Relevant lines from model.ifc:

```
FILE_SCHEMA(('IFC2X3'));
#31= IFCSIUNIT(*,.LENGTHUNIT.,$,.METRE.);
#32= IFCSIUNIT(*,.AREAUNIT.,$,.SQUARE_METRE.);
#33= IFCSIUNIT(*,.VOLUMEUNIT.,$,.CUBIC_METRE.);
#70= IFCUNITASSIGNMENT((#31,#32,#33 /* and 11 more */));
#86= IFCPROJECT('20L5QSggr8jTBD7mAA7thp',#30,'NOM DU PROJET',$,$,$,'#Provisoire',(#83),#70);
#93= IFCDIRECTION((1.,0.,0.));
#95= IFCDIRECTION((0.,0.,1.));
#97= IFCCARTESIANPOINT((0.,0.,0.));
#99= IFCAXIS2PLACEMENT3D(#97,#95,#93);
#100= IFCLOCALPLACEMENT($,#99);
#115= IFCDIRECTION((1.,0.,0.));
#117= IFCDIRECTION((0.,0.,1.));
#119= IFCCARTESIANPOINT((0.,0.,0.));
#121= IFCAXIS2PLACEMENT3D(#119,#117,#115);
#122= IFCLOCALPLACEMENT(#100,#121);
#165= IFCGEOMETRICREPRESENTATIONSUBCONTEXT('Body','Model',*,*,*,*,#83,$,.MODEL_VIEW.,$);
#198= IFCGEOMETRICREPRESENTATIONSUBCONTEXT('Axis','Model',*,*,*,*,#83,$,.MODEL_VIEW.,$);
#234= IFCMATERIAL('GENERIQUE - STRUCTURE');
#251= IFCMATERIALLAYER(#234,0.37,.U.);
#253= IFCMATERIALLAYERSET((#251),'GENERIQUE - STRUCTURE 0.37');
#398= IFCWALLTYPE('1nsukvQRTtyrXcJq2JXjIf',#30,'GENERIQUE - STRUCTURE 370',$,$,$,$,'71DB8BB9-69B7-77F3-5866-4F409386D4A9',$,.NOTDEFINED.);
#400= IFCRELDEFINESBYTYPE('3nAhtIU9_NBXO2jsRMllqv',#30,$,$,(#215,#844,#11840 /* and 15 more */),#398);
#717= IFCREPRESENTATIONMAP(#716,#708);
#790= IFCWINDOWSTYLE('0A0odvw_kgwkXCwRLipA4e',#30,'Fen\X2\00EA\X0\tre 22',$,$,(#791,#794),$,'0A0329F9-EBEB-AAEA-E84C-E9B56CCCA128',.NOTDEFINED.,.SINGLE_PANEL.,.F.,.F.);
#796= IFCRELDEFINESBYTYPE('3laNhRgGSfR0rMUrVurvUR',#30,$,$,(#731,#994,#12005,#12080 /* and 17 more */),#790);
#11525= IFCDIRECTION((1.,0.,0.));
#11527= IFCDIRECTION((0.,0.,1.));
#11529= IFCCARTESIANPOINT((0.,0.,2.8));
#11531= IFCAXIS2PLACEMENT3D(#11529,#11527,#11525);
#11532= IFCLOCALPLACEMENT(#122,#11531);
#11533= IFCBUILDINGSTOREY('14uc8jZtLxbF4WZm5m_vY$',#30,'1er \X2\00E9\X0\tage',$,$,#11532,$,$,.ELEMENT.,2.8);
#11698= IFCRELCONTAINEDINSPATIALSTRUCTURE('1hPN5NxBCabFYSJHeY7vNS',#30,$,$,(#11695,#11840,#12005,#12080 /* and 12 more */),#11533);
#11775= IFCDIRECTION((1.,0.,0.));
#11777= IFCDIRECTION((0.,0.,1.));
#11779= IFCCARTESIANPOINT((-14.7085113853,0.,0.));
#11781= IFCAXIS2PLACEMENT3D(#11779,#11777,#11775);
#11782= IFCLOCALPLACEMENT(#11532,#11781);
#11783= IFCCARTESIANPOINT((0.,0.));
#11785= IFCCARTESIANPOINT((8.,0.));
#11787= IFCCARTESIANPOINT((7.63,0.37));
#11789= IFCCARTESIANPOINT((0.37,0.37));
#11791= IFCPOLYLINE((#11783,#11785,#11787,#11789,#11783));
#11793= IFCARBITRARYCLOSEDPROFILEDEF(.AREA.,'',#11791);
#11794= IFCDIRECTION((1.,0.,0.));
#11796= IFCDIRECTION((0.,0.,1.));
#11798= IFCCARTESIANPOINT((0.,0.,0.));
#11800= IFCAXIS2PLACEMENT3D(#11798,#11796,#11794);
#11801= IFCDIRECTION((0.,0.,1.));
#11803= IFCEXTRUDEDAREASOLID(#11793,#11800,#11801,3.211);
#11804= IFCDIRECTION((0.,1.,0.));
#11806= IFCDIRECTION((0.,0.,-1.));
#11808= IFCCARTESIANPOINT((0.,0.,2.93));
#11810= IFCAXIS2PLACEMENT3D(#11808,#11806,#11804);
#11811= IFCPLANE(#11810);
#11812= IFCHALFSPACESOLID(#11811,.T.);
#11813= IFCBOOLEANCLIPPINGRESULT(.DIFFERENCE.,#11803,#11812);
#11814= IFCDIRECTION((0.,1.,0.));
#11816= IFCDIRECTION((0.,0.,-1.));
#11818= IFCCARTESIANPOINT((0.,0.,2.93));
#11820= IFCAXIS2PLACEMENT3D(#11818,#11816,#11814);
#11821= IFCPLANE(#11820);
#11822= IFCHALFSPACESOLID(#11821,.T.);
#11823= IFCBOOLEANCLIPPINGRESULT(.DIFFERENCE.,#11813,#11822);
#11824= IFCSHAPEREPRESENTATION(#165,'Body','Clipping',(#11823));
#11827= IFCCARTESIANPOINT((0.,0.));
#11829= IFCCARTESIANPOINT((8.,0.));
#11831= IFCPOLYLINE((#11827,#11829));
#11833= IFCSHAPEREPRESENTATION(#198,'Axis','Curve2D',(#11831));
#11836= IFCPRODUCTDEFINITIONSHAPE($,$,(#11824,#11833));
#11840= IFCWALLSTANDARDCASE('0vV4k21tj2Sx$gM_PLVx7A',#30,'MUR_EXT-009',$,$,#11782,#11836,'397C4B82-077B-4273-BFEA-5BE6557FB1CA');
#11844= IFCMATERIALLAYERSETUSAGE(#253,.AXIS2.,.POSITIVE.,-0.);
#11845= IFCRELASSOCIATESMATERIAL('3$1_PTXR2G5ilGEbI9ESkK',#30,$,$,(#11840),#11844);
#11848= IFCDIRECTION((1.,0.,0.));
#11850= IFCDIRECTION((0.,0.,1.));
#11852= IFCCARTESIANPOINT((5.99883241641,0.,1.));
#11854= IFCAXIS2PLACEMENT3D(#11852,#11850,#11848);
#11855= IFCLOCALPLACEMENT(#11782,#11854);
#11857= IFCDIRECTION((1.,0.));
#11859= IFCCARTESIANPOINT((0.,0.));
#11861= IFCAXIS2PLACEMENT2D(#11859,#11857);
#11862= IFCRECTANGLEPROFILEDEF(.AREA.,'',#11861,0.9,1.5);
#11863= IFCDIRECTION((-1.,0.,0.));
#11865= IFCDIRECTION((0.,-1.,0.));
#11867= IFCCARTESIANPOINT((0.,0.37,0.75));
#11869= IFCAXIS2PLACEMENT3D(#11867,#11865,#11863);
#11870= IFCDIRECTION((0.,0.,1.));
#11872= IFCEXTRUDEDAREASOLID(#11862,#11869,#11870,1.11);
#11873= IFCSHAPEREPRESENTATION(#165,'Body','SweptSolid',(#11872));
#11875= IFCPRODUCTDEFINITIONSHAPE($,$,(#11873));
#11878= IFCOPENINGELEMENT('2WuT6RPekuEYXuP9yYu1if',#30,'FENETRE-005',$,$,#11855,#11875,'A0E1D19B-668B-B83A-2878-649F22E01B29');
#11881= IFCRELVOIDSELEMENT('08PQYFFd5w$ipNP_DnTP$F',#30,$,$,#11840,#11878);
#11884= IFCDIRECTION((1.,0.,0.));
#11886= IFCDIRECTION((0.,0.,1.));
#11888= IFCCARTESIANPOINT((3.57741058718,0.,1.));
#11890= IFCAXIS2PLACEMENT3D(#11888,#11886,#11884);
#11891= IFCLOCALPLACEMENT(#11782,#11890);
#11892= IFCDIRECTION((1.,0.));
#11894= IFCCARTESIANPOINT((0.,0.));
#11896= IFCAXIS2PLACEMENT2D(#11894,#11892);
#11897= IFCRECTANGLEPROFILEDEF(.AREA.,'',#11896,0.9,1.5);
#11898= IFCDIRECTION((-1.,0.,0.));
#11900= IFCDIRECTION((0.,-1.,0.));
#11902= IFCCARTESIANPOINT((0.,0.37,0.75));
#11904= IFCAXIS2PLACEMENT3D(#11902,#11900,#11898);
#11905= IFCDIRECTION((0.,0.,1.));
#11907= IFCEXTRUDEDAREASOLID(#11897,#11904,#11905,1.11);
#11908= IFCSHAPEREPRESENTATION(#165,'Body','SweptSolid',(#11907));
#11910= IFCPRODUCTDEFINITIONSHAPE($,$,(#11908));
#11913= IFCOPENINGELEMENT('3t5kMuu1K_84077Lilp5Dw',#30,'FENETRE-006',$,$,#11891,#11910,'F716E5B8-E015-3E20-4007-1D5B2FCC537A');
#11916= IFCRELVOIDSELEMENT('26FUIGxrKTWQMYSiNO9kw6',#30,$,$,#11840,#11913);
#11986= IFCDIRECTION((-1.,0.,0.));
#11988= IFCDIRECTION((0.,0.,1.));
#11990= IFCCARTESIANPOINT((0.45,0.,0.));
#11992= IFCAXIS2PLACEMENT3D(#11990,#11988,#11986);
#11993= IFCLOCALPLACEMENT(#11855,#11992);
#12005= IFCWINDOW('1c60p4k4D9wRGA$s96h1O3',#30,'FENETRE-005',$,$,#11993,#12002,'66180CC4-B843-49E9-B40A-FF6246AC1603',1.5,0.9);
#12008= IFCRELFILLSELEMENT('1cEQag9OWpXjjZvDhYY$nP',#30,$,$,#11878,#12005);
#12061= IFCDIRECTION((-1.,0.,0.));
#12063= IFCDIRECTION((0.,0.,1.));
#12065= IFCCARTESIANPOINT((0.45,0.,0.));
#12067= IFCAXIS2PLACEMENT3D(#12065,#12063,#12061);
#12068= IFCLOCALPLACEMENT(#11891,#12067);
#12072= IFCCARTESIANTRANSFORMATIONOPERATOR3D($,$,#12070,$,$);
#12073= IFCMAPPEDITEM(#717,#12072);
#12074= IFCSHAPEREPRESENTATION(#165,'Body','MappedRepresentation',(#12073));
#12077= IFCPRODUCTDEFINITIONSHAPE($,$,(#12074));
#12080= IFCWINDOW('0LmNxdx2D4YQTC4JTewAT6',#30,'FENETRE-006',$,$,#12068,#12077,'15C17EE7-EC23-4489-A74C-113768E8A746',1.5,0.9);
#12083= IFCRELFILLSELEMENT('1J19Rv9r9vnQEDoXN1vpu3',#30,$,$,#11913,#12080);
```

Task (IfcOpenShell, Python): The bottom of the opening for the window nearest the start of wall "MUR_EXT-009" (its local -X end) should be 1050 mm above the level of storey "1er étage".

```python
import numpy as np
import ifcopenshell
import ifcopenshell.api.geometry
import ifcopenshell.geom
import ifcopenshell.util.element
import ifcopenshell.util.placement
import ifcopenshell.util.shape
import ifcopenshell.util.unit

model = ifcopenshell.open("model.ifc")
unit_scale = ifcopenshell.util.unit.calculate_unit_scale(model)

window = model.by_id(12080)
opening = window.FillsVoids[0].RelatingOpeningElement
storey = ifcopenshell.util.element.get_container(window, ifc_class="IfcBuildingStorey")
level = ifcopenshell.util.placement.get_local_placement(storey.ObjectPlacement)[2, 3]

# The opening's origin need not be at the sill, so measure its lowest point.
shape = ifcopenshell.geom.create_shape(ifcopenshell.geom.settings(), opening)
bottom = ifcopenshell.util.shape.get_shape_bottom_elevation(shape, shape.geometry) / unit_scale
dz = level + 1.05 / unit_scale - bottom

shift = np.array([0.0, 0.0, dz])
# The window is placed relative to its opening, so it follows when the opening moves.
matrix = ifcopenshell.util.placement.get_local_placement(opening.ObjectPlacement)
matrix[:3, 3] += shift
ifcopenshell.api.geometry.edit_object_placement(
    model, product=opening, matrix=matrix, is_si=False, should_transform_children=True
)

print(f"moved by {dz * unit_scale:+.3f} m")

model.write("model_edited.ifc")
```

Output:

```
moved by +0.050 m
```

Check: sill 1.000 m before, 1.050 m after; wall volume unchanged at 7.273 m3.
